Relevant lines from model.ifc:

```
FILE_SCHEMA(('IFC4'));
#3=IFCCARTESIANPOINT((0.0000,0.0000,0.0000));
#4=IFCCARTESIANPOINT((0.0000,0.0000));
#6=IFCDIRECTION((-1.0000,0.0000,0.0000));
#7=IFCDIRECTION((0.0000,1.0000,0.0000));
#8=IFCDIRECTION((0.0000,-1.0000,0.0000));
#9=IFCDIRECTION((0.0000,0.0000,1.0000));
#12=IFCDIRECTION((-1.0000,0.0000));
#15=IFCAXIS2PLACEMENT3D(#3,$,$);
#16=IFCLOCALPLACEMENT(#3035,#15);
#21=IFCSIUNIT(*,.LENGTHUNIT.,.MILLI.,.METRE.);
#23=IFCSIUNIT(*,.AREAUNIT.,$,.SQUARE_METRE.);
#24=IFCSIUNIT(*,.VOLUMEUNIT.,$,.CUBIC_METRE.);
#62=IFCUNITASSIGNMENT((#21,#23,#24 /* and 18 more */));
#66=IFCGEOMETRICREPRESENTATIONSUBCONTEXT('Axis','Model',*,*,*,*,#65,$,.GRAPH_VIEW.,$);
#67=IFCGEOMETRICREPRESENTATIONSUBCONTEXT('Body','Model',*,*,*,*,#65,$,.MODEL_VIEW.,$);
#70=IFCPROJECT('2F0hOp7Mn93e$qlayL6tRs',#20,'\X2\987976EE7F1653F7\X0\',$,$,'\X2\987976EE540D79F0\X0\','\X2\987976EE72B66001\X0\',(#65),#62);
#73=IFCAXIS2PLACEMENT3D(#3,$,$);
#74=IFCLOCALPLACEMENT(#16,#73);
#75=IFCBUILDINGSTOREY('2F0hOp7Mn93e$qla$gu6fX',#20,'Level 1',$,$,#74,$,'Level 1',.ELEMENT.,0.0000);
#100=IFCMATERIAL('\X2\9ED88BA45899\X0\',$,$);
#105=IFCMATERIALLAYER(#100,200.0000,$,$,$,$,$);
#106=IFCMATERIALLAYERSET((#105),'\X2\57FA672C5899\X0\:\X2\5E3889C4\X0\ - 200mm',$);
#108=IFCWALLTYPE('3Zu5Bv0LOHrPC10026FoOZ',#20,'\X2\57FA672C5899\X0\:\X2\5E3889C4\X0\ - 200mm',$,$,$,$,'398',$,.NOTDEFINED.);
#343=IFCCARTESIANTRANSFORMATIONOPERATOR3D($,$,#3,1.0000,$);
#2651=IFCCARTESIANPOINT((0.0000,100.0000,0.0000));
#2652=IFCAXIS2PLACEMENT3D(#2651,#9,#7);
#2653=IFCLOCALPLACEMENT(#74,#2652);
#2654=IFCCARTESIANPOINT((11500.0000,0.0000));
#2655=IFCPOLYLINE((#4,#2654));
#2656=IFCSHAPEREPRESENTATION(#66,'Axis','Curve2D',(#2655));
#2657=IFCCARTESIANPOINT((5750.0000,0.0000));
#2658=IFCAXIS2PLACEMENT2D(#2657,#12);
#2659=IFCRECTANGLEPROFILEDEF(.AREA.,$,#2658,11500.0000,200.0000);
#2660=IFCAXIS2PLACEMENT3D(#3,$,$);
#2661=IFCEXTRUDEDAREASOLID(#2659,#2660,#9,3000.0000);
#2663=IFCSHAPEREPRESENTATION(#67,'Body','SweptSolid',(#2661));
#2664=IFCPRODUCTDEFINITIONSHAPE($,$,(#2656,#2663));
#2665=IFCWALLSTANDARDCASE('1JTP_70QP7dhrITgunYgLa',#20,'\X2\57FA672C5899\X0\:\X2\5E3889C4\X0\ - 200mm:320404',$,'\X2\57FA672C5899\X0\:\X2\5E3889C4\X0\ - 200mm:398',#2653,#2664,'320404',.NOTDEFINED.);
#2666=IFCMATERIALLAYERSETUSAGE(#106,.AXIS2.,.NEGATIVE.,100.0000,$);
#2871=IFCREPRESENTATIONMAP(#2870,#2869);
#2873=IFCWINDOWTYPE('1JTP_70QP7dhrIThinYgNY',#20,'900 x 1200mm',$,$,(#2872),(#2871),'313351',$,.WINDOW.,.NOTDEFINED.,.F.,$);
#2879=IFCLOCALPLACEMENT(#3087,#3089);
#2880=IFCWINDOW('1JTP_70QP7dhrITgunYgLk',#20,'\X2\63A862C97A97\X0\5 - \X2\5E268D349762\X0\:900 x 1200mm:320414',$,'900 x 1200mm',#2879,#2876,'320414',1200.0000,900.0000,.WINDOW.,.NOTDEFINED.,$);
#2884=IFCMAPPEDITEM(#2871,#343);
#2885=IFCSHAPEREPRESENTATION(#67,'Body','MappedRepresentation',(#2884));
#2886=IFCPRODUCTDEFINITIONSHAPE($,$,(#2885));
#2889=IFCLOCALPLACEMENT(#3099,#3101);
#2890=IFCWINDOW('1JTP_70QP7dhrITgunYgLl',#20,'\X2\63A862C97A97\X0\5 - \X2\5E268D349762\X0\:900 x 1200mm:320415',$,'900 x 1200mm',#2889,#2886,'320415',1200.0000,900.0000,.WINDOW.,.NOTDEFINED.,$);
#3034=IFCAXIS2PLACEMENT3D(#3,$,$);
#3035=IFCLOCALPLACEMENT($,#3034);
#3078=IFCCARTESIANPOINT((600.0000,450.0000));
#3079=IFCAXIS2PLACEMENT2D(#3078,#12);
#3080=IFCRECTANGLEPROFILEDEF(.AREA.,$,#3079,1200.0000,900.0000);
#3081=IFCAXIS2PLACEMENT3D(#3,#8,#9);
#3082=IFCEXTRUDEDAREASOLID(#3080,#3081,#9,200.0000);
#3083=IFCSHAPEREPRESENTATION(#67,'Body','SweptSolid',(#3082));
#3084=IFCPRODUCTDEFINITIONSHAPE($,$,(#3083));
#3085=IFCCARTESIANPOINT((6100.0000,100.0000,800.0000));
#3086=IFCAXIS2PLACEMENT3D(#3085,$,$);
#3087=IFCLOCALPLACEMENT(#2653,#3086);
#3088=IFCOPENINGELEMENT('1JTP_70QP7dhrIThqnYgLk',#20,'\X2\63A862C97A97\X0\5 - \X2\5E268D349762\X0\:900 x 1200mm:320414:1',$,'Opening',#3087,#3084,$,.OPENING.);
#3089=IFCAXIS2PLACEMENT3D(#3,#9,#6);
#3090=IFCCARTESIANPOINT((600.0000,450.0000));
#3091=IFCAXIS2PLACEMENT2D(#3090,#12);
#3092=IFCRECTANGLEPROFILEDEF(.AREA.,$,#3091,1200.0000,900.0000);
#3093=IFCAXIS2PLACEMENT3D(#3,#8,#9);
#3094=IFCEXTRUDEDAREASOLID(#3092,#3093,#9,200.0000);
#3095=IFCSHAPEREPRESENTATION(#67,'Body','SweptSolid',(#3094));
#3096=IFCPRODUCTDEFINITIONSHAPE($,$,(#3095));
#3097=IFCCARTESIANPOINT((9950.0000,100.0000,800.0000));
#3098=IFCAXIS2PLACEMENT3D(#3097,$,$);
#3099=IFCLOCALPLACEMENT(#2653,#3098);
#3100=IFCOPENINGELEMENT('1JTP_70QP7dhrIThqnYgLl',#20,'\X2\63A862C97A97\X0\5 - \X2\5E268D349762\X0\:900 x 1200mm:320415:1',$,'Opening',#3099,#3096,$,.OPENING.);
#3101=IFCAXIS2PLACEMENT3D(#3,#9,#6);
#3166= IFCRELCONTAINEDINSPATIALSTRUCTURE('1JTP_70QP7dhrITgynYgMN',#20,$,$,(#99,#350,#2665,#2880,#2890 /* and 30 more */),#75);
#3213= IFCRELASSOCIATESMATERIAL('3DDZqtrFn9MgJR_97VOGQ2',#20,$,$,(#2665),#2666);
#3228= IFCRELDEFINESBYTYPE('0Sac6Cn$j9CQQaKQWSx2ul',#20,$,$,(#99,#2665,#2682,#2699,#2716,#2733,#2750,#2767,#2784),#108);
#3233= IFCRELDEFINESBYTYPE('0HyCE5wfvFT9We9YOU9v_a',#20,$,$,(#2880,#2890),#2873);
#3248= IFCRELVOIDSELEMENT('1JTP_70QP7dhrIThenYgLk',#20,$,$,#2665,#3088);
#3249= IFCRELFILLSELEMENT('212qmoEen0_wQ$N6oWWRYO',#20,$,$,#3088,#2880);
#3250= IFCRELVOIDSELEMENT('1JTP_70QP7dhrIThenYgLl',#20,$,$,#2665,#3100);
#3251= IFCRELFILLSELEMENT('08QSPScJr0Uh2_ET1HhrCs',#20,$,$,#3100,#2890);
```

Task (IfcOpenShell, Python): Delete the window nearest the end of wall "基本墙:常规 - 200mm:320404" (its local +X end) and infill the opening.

```python
import ifcopenshell
import ifcopenshell.api.feature
import ifcopenshell.api.root
import ifcopenshell.geom
import ifcopenshell.util.shape

model = ifcopenshell.open("model.ifc")
settings = ifcopenshell.geom.settings()


def volume(element):
    """Net volume in cubic metres, openings subtracted."""
    shape = ifcopenshell.geom.create_shape(settings, element)
    return ifcopenshell.util.shape.get_volume(shape.geometry)


window = model.by_id(2890)
opening = window.FillsVoids[0].RelatingOpeningElement
wall = opening.VoidsElements[0].RelatingBuildingElement
before = volume(wall)

ifcopenshell.api.root.remove_product(model, product=window)
ifcopenshell.api.feature.remove_feature(model, feature=opening)

after = volume(wall)

print(f"wall volume {before:.3f} -> {after:.3f} m3")

model.write("model_updated.ifc")
```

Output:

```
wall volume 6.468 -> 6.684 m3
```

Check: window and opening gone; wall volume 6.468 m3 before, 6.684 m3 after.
